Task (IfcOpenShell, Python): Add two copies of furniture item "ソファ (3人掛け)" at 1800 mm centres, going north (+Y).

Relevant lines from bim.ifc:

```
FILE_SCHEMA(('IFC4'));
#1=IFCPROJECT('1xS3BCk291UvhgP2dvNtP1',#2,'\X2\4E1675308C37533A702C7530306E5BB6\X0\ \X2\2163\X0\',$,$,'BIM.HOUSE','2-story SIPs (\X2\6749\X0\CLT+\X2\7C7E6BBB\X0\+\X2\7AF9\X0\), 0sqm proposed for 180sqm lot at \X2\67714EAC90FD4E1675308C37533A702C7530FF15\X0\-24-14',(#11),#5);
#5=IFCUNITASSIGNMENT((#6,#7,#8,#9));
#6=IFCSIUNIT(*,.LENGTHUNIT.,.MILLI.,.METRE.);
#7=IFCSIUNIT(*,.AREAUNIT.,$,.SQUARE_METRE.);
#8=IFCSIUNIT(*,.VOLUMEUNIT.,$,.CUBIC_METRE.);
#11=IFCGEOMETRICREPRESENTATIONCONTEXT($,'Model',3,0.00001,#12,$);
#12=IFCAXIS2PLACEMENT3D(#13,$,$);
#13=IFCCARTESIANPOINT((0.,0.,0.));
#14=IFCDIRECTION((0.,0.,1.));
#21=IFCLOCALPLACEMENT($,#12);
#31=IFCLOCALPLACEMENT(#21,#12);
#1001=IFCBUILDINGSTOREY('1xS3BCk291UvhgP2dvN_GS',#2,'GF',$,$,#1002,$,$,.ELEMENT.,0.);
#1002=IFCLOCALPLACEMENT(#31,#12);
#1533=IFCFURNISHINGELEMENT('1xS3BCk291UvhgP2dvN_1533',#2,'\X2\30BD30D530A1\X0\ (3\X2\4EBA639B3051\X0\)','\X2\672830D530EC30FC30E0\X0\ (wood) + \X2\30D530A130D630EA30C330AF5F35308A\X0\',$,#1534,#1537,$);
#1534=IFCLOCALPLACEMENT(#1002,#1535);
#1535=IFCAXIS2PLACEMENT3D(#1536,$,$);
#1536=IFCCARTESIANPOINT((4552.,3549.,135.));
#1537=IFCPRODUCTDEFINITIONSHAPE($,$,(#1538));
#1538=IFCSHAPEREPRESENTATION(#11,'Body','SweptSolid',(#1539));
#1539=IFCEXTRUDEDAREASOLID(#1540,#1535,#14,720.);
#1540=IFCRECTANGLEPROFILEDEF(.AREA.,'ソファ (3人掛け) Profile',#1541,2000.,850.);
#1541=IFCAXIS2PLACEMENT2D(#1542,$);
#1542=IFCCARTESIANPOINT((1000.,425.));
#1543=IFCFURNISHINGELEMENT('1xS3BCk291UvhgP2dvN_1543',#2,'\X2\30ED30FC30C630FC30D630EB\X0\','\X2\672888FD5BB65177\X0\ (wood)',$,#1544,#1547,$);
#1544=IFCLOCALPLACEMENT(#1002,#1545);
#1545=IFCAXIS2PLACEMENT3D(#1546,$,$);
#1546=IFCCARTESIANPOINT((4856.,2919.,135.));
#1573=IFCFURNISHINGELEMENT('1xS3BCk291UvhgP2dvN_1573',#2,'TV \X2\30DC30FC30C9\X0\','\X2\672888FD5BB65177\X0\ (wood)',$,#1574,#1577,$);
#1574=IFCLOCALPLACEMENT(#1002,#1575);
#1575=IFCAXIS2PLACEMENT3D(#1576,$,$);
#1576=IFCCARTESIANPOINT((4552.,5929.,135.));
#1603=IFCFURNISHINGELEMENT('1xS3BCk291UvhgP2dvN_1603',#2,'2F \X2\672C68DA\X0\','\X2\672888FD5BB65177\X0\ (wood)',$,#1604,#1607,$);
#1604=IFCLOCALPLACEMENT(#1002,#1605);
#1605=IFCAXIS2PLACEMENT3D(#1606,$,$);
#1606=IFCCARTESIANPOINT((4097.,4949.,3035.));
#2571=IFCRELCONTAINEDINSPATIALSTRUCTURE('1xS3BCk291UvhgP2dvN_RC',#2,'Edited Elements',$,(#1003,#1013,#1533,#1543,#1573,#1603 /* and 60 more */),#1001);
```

```python
import numpy as np
import ifcopenshell
import ifcopenshell.api.geometry
import ifcopenshell.api.root
import ifcopenshell.util.element
import ifcopenshell.util.placement
import ifcopenshell.util.unit

model = ifcopenshell.open("bim.ifc")
unit_scale = ifcopenshell.util.unit.calculate_unit_scale(model)


def reuse_history(source, copy):
    """copy_class also copies each property set's owner history, people and application; keep the originals."""
    for rel in copy.IsDefinedBy:
        if rel.is_a("IfcRelDefinesByProperties") and (history := rel.RelatingPropertyDefinition.OwnerHistory):
            rel.RelatingPropertyDefinition.OwnerHistory = source.OwnerHistory
            ifcopenshell.util.element.remove_deep2(model, history)


source = model.by_guid("1xS3BCk291UvhgP2dvN_1533")
base = ifcopenshell.util.placement.get_local_placement(source.ObjectPlacement)
step = np.array([0.0, 1.0, 0.0]) * 1.8 / unit_scale

for i in range(1, 3):
    copy = ifcopenshell.api.root.copy_class(model, product=source)
    copy.Representation = ifcopenshell.util.element.copy_deep(
        model, source.Representation, exclude=["IfcGeometricRepresentationContext", "IfcRepresentationMap"]
    )
    reuse_history(source, copy)
    matrix = base.copy()
    matrix[:3, 3] += i * step
    print("added at", matrix[:3, 3].round(3) + 0.0)
    ifcopenshell.api.geometry.edit_object_placement(model, product=copy, matrix=matrix, is_si=False)

model.write("bim_edited.ifc")
```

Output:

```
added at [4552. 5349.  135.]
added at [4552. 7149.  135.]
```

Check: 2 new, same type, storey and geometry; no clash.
